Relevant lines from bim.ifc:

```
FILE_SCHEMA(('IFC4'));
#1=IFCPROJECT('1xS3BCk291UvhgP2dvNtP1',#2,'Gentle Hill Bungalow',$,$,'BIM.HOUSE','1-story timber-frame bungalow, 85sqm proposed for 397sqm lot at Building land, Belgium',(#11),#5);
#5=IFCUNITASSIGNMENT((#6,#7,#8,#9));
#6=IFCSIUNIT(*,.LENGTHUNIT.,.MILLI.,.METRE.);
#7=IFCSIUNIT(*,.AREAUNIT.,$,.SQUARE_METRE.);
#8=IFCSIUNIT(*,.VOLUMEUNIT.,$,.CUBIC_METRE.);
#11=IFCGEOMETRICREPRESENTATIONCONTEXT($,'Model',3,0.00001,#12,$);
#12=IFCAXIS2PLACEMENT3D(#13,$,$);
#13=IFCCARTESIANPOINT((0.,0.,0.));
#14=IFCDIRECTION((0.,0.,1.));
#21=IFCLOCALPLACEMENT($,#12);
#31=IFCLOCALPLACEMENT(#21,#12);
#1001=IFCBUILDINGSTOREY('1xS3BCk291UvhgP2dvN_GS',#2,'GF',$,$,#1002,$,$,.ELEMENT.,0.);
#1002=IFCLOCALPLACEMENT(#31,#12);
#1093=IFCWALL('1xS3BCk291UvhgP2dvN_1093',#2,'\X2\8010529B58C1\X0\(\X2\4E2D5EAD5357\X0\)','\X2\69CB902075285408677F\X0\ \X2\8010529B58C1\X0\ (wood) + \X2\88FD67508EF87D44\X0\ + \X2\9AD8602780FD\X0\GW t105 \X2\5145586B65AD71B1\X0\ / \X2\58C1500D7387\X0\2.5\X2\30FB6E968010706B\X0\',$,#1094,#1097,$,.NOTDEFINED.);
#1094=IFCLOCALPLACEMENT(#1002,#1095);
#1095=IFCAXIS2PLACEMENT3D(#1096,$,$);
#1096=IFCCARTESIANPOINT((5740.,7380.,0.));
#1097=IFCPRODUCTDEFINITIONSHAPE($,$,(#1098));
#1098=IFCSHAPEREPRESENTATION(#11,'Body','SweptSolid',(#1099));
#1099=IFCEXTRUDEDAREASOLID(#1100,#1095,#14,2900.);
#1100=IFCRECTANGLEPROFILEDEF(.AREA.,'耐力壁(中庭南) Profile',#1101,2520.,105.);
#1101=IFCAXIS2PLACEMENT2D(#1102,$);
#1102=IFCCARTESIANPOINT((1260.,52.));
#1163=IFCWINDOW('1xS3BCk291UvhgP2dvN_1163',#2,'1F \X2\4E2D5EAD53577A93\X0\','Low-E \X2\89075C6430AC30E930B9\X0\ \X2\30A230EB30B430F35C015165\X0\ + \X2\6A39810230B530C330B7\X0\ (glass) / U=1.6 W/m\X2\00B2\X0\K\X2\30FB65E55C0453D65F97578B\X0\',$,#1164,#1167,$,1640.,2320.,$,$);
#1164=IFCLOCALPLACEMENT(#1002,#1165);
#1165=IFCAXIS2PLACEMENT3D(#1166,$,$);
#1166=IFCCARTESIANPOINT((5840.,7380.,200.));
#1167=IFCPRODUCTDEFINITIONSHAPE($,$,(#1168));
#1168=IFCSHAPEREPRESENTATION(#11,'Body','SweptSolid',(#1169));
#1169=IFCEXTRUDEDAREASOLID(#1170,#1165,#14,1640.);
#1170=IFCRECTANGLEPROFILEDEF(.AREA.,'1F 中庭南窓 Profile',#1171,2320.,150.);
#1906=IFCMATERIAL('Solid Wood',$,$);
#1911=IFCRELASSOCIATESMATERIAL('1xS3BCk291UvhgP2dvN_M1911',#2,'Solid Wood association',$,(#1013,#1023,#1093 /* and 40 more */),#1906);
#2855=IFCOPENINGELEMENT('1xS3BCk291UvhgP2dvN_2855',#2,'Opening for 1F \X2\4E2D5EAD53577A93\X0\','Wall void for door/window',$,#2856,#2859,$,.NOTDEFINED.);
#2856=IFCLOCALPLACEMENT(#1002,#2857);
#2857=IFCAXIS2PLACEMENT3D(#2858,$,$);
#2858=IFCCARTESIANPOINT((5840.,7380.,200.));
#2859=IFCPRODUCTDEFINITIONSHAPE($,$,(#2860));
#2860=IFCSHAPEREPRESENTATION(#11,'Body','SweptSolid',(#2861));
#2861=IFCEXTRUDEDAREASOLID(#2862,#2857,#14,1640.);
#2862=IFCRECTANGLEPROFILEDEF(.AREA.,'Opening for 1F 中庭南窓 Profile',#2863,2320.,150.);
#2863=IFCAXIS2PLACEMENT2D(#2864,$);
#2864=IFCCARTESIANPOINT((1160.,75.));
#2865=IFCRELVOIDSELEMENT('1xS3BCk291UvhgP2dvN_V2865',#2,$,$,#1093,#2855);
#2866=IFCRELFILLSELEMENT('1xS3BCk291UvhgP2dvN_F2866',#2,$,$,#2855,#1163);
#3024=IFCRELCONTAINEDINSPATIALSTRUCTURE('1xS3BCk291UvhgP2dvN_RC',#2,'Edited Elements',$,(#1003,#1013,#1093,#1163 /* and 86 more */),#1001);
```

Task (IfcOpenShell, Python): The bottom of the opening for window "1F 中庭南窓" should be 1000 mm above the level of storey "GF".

```python
import numpy as np
import ifcopenshell
import ifcopenshell.api.geometry
import ifcopenshell.geom
import ifcopenshell.util.element
import ifcopenshell.util.placement
import ifcopenshell.util.shape
import ifcopenshell.util.unit

model = ifcopenshell.open("bim.ifc")
unit_scale = ifcopenshell.util.unit.calculate_unit_scale(model)

window = model.by_guid("1xS3BCk291UvhgP2dvN_1163")
opening = window.FillsVoids[0].RelatingOpeningElement
storey = ifcopenshell.util.element.get_container(window, ifc_class="IfcBuildingStorey")
level = ifcopenshell.util.placement.get_local_placement(storey.ObjectPlacement)[2, 3]

# The opening's origin need not be at the sill, so measure its lowest point.
shape = ifcopenshell.geom.create_shape(ifcopenshell.geom.settings(), opening)
bottom = ifcopenshell.util.shape.get_shape_bottom_elevation(shape, shape.geometry) / unit_scale
dz = level + 1000.0 - bottom

shift = np.array([0.0, 0.0, dz])
# The window is not placed relative to its opening, so move both.
for product in (opening, window):
    matrix = ifcopenshell.util.placement.get_local_placement(product.ObjectPlacement)
    matrix[:3, 3] += shift
    ifcopenshell.api.geometry.edit_object_placement(model, product=product, matrix=matrix, is_si=False)

print(f"moved by {dz * unit_scale:+.3f} m")

model.write("bim-out.ifc")
```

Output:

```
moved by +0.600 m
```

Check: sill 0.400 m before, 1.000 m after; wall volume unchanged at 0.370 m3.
